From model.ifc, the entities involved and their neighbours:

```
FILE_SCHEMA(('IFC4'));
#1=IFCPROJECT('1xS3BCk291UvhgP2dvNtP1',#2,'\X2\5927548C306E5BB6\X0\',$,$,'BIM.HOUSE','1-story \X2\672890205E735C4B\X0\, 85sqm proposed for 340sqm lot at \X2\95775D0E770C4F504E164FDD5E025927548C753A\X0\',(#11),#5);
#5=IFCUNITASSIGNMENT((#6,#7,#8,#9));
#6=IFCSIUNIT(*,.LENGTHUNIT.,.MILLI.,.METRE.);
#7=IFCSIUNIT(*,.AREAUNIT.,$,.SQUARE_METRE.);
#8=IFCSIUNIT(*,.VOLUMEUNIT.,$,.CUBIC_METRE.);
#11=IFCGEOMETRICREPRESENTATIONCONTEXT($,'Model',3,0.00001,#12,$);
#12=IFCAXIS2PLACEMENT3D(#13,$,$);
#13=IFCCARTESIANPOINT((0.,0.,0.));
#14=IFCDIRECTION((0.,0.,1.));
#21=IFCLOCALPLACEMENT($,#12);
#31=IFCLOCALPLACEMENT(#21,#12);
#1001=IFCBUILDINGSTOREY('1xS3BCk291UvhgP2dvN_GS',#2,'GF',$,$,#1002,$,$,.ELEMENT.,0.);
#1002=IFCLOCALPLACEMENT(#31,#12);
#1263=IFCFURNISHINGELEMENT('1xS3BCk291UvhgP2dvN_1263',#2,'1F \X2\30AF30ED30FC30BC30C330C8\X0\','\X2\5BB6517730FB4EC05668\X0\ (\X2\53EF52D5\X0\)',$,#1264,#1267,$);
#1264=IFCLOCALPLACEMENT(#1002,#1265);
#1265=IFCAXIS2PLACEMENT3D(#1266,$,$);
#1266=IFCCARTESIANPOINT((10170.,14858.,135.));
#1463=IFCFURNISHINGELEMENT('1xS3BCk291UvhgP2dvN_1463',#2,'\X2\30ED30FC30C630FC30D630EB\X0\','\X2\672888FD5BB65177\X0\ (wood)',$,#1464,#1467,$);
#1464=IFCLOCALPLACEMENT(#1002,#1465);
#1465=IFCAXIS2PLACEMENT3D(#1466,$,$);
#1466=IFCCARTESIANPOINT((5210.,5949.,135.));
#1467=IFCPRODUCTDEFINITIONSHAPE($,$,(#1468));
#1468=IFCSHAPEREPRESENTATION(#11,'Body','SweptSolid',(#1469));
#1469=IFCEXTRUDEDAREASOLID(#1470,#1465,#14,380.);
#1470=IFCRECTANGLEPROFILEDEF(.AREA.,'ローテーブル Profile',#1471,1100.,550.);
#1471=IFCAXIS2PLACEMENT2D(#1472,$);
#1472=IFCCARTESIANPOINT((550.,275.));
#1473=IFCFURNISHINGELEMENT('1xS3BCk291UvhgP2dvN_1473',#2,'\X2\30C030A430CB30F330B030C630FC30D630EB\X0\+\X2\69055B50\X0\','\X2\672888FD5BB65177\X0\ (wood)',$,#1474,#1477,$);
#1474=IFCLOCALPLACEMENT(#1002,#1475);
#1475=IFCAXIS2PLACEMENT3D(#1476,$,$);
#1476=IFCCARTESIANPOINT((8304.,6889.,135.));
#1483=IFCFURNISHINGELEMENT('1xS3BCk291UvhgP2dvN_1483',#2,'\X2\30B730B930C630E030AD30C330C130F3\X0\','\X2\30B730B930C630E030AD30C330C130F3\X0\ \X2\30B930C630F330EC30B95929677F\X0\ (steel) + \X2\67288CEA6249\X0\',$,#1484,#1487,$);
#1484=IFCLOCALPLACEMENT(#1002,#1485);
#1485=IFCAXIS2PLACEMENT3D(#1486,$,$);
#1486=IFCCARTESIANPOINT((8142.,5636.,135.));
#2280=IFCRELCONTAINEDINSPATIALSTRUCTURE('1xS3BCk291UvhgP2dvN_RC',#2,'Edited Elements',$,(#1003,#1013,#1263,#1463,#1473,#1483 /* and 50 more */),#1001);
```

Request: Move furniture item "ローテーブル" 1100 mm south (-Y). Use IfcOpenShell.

```python
import ifcopenshell
import ifcopenshell.api.geometry
import ifcopenshell.util.placement
import ifcopenshell.util.unit

model = ifcopenshell.open("model.ifc")
unit_scale = ifcopenshell.util.unit.calculate_unit_scale(model)

item = model.by_guid("1xS3BCk291UvhgP2dvN_1463")
matrix = ifcopenshell.util.placement.get_local_placement(item.ObjectPlacement)
matrix[1, 3] -= 1.1 / unit_scale
ifcopenshell.api.geometry.edit_object_placement(model, product=item, matrix=matrix, is_si=False)

print(ifcopenshell.util.placement.get_local_placement(item.ObjectPlacement).round(3) + 0.0)

model.write("model-out.ifc")
```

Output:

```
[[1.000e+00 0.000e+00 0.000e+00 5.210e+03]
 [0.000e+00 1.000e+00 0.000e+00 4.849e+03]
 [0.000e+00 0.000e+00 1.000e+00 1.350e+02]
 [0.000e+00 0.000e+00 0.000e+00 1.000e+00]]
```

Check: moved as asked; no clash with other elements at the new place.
